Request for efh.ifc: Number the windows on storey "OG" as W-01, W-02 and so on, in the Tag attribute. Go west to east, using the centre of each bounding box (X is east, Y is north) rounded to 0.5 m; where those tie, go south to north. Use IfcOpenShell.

First a look at what the model holds.

```python
import ifcopenshell
import ifcopenshell.util.element
import ifcopenshell.util.placement

model = ifcopenshell.open("efh.ifc")
print(model.schema)
storey = next(s for s in model.by_type("IfcBuildingStorey") if s.Name == "OG")
windows = [e for e in ifcopenshell.util.element.get_decomposition(storey) if e.is_a("IfcWindow")]
for e in sorted(windows, key=lambda e: e.id()):
    origin = ifcopenshell.util.placement.get_local_placement(e.ObjectPlacement)[:3, 3]
    print(e.id(), e.Tag, e.Name, origin.round(2) + 0.0, sep=" | ")
```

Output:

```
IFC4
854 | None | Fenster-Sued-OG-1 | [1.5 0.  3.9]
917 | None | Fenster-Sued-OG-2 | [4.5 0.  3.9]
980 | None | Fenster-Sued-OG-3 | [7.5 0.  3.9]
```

```python
import ifcopenshell
import ifcopenshell.geom
import ifcopenshell.util.element
import ifcopenshell.util.shape

model = ifcopenshell.open("efh.ifc")
settings = ifcopenshell.geom.settings()
settings.set("use-world-coords", True)


def centre(element):
    shape = ifcopenshell.geom.create_shape(settings, element)
    return ifcopenshell.util.shape.get_bbox_centroid(shape.geometry)


storey = next(s for s in model.by_type("IfcBuildingStorey") if s.Name == "OG")
windows = [e for e in ifcopenshell.util.element.get_decomposition(storey) if e.is_a("IfcWindow")]

# Insertion points can sit at a corner or the storey origin, so sort by the geometry (in metres).
centres = {e: centre(e) for e in windows}
windows.sort(key=lambda e: (round(centres[e][0] / 0.5), centres[e][1]))

for i, e in enumerate(windows, start=1):
    number = f"W-{i:02d}"
    e.Tag = number
    print(e.id(), number)

model.write("efh_edited.ifc")
```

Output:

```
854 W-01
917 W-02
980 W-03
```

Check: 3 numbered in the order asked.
